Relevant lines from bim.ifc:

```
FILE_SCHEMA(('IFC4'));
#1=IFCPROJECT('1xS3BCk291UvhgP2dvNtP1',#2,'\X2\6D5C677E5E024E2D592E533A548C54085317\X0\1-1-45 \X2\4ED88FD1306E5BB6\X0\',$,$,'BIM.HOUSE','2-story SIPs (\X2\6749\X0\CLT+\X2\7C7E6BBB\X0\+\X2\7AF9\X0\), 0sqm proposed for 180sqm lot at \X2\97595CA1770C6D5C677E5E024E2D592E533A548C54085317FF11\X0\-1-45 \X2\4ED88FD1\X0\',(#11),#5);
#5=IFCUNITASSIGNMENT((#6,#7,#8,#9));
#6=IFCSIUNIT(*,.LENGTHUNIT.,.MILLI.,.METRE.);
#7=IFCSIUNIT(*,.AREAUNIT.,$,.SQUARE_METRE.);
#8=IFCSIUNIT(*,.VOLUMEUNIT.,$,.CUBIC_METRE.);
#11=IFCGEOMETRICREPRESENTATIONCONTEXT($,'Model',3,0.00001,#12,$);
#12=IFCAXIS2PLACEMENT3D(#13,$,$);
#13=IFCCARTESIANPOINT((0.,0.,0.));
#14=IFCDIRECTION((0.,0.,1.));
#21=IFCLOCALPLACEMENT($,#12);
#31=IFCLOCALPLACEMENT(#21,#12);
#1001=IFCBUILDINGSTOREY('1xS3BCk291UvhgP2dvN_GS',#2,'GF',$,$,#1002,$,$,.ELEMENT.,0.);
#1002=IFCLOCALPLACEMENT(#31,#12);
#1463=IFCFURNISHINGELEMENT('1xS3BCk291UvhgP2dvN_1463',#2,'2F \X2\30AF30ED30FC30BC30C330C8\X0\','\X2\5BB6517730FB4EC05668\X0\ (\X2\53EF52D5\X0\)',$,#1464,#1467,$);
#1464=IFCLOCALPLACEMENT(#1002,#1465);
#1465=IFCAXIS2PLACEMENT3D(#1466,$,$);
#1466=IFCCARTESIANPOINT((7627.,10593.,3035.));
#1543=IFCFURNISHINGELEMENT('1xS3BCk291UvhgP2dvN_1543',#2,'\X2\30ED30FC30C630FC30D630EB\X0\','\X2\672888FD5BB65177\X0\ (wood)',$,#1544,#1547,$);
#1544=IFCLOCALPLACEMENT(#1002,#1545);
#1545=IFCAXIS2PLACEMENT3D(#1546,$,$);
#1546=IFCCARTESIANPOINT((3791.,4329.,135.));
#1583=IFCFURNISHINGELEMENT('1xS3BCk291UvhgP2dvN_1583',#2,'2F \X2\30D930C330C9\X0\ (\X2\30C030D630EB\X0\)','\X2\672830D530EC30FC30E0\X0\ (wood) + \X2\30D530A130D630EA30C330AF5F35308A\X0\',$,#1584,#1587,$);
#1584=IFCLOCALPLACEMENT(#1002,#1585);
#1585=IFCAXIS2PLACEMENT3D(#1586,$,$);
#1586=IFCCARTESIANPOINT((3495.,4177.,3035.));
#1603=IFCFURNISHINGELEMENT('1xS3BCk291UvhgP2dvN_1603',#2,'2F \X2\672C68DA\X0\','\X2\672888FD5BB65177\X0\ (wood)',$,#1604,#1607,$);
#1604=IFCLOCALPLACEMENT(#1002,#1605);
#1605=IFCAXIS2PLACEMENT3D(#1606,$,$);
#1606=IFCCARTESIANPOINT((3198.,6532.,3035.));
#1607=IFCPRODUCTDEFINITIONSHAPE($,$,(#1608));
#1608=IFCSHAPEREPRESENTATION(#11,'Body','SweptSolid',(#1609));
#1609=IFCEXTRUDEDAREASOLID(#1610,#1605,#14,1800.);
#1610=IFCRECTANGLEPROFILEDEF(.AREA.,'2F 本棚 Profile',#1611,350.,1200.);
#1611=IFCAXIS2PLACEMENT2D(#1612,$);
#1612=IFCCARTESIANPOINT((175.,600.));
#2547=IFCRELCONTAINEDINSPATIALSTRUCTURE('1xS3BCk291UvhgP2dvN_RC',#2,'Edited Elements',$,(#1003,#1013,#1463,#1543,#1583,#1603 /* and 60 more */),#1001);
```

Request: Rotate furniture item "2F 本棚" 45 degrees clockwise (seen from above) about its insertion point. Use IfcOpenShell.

```python
import ifcopenshell
import ifcopenshell.api.geometry
import ifcopenshell.util.placement

model = ifcopenshell.open("bim.ifc")

item = model.by_guid("1xS3BCk291UvhgP2dvN_1603")
matrix = ifcopenshell.util.placement.get_local_placement(item.ObjectPlacement)
matrix = matrix @ ifcopenshell.util.placement.rotation(-45, "Z")
ifcopenshell.api.geometry.edit_object_placement(model, product=item, matrix=matrix, is_si=False)

print(ifcopenshell.util.placement.get_local_placement(item.ObjectPlacement).round(3) + 0.0)

model.write("bim_edited.ifc")
```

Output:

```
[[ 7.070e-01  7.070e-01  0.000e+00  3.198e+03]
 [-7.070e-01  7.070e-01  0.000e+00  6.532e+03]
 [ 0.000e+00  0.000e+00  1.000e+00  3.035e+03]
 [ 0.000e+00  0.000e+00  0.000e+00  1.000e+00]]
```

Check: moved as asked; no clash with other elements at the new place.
